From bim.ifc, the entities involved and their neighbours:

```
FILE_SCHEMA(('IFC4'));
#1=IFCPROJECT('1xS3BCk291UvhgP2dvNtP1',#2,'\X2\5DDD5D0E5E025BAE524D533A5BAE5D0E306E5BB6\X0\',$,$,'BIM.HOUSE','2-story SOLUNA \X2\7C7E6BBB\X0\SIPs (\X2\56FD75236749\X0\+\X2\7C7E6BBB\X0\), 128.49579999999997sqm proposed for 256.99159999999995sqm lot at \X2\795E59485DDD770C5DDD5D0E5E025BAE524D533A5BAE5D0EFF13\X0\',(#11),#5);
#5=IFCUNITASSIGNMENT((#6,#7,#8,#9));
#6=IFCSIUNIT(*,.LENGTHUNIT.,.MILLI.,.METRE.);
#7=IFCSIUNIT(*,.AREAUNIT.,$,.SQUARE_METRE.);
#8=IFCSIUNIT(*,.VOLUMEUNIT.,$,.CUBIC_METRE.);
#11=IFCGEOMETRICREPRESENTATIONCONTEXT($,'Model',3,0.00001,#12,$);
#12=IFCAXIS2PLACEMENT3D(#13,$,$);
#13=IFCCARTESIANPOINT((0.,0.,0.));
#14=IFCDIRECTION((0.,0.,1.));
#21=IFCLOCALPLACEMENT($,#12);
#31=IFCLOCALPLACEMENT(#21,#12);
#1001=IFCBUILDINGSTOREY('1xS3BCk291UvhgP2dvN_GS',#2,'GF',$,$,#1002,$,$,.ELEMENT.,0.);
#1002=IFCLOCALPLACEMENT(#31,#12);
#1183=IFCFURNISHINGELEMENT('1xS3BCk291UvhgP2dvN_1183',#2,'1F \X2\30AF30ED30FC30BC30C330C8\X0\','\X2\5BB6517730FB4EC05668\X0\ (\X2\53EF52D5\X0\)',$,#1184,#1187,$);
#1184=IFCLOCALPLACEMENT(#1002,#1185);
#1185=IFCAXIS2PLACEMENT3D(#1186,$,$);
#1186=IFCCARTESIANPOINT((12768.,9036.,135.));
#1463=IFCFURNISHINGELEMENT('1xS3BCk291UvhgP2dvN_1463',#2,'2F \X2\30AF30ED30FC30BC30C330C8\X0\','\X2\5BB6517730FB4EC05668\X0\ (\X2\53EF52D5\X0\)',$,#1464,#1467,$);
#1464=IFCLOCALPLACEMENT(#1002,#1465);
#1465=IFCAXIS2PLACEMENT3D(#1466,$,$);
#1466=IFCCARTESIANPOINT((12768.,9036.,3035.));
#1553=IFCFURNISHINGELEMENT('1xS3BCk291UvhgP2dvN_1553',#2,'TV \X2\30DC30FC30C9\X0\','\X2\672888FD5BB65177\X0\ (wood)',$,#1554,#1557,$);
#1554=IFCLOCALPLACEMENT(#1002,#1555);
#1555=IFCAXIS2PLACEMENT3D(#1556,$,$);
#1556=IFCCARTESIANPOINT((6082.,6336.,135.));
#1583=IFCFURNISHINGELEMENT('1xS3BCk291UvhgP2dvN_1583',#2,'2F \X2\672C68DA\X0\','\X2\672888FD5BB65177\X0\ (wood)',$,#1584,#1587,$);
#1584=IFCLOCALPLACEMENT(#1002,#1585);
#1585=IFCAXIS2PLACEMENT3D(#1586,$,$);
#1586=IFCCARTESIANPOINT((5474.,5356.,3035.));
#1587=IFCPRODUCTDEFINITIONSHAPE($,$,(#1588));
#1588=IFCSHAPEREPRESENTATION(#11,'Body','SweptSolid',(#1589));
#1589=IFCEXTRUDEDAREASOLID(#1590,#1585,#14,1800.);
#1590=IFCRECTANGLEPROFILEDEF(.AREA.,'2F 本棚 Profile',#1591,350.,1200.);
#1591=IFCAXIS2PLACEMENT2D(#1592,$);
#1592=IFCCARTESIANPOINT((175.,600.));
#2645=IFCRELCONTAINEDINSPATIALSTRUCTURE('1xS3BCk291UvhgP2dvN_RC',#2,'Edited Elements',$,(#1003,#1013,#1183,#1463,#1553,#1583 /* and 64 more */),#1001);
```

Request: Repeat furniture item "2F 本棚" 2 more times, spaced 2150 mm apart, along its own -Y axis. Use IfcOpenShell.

```python
import ifcopenshell
import ifcopenshell.api.geometry
import ifcopenshell.api.root
import ifcopenshell.util.element
import ifcopenshell.util.placement

model = ifcopenshell.open("bim.ifc")


def reuse_history(source, copy):
    """copy_class also copies each property set's owner history, people and application; keep the originals."""
    for rel in copy.IsDefinedBy:
        if rel.is_a("IfcRelDefinesByProperties") and (history := rel.RelatingPropertyDefinition.OwnerHistory):
            rel.RelatingPropertyDefinition.OwnerHistory = source.OwnerHistory
            ifcopenshell.util.element.remove_deep2(model, history)


source = model.by_id(1583)
base = ifcopenshell.util.placement.get_local_placement(source.ObjectPlacement)
step = -base[:3, 1] * 2150.0

for i in range(1, 3):
    copy = ifcopenshell.api.root.copy_class(model, product=source)
    copy.Representation = ifcopenshell.util.element.copy_deep(
        model, source.Representation, exclude=["IfcGeometricRepresentationContext", "IfcRepresentationMap"]
    )
    reuse_history(source, copy)
    matrix = base.copy()
    matrix[:3, 3] += i * step
    print("added at", matrix[:3, 3].round(3) + 0.0)
    ifcopenshell.api.geometry.edit_object_placement(model, product=copy, matrix=matrix, is_si=False)

model.write("bim-out.ifc")
```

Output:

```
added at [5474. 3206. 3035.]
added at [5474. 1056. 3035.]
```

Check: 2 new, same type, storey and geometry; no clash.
